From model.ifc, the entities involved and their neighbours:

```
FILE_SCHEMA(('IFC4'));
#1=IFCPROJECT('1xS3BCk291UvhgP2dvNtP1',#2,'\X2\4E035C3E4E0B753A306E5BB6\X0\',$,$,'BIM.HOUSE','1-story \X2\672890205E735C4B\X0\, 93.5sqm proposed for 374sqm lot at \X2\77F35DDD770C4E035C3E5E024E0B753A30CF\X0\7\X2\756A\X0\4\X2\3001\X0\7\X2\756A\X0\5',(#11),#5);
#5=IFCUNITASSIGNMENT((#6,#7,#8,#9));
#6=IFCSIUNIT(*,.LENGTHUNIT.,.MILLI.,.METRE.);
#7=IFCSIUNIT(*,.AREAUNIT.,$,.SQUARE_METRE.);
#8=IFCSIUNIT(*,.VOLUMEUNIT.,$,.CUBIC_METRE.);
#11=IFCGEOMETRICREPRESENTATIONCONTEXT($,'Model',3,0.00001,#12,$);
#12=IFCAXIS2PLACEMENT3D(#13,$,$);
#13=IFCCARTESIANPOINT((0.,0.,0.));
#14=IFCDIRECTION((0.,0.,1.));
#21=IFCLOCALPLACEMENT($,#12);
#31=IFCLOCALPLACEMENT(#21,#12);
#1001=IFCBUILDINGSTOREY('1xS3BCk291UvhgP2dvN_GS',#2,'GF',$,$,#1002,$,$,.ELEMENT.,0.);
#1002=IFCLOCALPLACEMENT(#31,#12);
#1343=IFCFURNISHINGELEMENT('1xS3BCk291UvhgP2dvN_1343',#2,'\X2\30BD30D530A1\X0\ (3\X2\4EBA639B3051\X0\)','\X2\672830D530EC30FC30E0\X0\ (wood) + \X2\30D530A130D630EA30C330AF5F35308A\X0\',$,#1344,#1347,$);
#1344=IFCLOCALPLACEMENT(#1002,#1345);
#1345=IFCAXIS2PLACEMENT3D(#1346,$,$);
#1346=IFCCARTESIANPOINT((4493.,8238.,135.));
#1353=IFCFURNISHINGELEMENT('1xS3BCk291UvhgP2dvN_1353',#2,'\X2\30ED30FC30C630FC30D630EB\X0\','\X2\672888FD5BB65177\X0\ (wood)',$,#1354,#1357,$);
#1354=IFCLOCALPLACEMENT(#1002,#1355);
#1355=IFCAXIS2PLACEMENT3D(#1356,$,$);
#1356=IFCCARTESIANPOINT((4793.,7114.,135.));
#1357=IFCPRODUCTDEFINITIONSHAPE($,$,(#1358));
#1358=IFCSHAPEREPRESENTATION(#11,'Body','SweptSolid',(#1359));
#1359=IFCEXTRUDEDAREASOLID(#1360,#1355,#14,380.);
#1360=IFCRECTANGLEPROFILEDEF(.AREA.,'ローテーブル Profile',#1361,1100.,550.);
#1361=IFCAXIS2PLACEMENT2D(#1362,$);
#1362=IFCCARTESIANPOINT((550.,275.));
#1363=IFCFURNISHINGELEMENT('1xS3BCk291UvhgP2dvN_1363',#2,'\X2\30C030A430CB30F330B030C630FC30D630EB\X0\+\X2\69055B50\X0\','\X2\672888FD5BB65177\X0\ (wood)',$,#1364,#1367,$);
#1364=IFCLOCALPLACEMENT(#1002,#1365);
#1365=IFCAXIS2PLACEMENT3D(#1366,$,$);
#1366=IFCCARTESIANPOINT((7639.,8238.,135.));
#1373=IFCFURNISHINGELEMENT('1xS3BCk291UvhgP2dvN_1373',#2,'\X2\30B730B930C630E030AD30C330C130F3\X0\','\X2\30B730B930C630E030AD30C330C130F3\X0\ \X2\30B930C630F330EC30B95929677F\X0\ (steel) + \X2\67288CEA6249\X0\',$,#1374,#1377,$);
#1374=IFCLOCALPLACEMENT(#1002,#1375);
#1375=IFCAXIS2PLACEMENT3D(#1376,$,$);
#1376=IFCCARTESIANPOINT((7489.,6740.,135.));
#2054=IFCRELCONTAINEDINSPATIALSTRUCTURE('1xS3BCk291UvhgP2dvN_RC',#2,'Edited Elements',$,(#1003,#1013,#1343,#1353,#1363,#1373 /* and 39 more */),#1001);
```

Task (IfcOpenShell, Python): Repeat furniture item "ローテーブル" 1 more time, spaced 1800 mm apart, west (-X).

```python
import numpy as np
import ifcopenshell
import ifcopenshell.api.geometry
import ifcopenshell.api.root
import ifcopenshell.util.element
import ifcopenshell.util.placement

model = ifcopenshell.open("model.ifc")


def reuse_history(source, copy):
    """copy_class also copies each property set's owner history, people and application; keep the originals."""
    for rel in copy.IsDefinedBy:
        if rel.is_a("IfcRelDefinesByProperties") and (history := rel.RelatingPropertyDefinition.OwnerHistory):
            rel.RelatingPropertyDefinition.OwnerHistory = source.OwnerHistory
            ifcopenshell.util.element.remove_deep2(model, history)


source = model.by_guid("1xS3BCk291UvhgP2dvN_1353")
base = ifcopenshell.util.placement.get_local_placement(source.ObjectPlacement)
step = np.array([-1.0, 0.0, 0.0]) * 1800.0

for i in range(1, 2):
    copy = ifcopenshell.api.root.copy_class(model, product=source)
    copy.Representation = ifcopenshell.util.element.copy_deep(
        model, source.Representation, exclude=["IfcGeometricRepresentationContext", "IfcRepresentationMap"]
    )
    reuse_history(source, copy)
    matrix = base.copy()
    matrix[:3, 3] += i * step
    print("added at", matrix[:3, 3].round(3) + 0.0)
    ifcopenshell.api.geometry.edit_object_placement(model, product=copy, matrix=matrix, is_si=False)

model.write("model_rev.ifc")
```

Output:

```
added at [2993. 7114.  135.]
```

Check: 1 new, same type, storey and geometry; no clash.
